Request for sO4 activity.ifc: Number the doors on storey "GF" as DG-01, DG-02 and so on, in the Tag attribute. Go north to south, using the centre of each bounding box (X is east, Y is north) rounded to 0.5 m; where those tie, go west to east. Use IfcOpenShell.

First a look at what the model holds.

```python
import ifcopenshell
import ifcopenshell.util.element
import ifcopenshell.util.placement

model = ifcopenshell.open("sO4 activity.ifc")
print(model.schema)
storey = next(s for s in model.by_type("IfcBuildingStorey") if s.Name == "GF")
doors = [e for e in ifcopenshell.util.element.get_decomposition(storey) if e.is_a("IfcDoor")]
for e in sorted(doors, key=lambda e: e.id()):
    origin = ifcopenshell.util.placement.get_local_placement(e.ObjectPlacement)[:3, 3]
    print(e.id(), e.Tag, e.Name, origin.round(2) + 0.0, sep=" | ")
```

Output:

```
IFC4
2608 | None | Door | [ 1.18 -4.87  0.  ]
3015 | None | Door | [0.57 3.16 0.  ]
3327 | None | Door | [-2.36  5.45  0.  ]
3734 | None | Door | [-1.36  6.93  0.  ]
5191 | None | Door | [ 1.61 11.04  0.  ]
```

```python
import ifcopenshell
import ifcopenshell.geom
import ifcopenshell.util.element
import ifcopenshell.util.shape

model = ifcopenshell.open("sO4 activity.ifc")
settings = ifcopenshell.geom.settings()
settings.set("use-world-coords", True)


def centre(element):
    shape = ifcopenshell.geom.create_shape(settings, element)
    return ifcopenshell.util.shape.get_bbox_centroid(shape.geometry)


storey = next(s for s in model.by_type("IfcBuildingStorey") if s.Name == "GF")
doors = [e for e in ifcopenshell.util.element.get_decomposition(storey) if e.is_a("IfcDoor")]

# Insertion points can sit at a corner or the storey origin, so sort by the geometry (in metres).
centres = {e: centre(e) for e in doors}
doors.sort(key=lambda e: (-round(centres[e][1] / 0.5), centres[e][0]))

for i, e in enumerate(doors, start=1):
    number = f"DG-{i:02d}"
    e.Tag = number
    print(e.id(), number)

model.write("sO4 activity_updated.ifc")
```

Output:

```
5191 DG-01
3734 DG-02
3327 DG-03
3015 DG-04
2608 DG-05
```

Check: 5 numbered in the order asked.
